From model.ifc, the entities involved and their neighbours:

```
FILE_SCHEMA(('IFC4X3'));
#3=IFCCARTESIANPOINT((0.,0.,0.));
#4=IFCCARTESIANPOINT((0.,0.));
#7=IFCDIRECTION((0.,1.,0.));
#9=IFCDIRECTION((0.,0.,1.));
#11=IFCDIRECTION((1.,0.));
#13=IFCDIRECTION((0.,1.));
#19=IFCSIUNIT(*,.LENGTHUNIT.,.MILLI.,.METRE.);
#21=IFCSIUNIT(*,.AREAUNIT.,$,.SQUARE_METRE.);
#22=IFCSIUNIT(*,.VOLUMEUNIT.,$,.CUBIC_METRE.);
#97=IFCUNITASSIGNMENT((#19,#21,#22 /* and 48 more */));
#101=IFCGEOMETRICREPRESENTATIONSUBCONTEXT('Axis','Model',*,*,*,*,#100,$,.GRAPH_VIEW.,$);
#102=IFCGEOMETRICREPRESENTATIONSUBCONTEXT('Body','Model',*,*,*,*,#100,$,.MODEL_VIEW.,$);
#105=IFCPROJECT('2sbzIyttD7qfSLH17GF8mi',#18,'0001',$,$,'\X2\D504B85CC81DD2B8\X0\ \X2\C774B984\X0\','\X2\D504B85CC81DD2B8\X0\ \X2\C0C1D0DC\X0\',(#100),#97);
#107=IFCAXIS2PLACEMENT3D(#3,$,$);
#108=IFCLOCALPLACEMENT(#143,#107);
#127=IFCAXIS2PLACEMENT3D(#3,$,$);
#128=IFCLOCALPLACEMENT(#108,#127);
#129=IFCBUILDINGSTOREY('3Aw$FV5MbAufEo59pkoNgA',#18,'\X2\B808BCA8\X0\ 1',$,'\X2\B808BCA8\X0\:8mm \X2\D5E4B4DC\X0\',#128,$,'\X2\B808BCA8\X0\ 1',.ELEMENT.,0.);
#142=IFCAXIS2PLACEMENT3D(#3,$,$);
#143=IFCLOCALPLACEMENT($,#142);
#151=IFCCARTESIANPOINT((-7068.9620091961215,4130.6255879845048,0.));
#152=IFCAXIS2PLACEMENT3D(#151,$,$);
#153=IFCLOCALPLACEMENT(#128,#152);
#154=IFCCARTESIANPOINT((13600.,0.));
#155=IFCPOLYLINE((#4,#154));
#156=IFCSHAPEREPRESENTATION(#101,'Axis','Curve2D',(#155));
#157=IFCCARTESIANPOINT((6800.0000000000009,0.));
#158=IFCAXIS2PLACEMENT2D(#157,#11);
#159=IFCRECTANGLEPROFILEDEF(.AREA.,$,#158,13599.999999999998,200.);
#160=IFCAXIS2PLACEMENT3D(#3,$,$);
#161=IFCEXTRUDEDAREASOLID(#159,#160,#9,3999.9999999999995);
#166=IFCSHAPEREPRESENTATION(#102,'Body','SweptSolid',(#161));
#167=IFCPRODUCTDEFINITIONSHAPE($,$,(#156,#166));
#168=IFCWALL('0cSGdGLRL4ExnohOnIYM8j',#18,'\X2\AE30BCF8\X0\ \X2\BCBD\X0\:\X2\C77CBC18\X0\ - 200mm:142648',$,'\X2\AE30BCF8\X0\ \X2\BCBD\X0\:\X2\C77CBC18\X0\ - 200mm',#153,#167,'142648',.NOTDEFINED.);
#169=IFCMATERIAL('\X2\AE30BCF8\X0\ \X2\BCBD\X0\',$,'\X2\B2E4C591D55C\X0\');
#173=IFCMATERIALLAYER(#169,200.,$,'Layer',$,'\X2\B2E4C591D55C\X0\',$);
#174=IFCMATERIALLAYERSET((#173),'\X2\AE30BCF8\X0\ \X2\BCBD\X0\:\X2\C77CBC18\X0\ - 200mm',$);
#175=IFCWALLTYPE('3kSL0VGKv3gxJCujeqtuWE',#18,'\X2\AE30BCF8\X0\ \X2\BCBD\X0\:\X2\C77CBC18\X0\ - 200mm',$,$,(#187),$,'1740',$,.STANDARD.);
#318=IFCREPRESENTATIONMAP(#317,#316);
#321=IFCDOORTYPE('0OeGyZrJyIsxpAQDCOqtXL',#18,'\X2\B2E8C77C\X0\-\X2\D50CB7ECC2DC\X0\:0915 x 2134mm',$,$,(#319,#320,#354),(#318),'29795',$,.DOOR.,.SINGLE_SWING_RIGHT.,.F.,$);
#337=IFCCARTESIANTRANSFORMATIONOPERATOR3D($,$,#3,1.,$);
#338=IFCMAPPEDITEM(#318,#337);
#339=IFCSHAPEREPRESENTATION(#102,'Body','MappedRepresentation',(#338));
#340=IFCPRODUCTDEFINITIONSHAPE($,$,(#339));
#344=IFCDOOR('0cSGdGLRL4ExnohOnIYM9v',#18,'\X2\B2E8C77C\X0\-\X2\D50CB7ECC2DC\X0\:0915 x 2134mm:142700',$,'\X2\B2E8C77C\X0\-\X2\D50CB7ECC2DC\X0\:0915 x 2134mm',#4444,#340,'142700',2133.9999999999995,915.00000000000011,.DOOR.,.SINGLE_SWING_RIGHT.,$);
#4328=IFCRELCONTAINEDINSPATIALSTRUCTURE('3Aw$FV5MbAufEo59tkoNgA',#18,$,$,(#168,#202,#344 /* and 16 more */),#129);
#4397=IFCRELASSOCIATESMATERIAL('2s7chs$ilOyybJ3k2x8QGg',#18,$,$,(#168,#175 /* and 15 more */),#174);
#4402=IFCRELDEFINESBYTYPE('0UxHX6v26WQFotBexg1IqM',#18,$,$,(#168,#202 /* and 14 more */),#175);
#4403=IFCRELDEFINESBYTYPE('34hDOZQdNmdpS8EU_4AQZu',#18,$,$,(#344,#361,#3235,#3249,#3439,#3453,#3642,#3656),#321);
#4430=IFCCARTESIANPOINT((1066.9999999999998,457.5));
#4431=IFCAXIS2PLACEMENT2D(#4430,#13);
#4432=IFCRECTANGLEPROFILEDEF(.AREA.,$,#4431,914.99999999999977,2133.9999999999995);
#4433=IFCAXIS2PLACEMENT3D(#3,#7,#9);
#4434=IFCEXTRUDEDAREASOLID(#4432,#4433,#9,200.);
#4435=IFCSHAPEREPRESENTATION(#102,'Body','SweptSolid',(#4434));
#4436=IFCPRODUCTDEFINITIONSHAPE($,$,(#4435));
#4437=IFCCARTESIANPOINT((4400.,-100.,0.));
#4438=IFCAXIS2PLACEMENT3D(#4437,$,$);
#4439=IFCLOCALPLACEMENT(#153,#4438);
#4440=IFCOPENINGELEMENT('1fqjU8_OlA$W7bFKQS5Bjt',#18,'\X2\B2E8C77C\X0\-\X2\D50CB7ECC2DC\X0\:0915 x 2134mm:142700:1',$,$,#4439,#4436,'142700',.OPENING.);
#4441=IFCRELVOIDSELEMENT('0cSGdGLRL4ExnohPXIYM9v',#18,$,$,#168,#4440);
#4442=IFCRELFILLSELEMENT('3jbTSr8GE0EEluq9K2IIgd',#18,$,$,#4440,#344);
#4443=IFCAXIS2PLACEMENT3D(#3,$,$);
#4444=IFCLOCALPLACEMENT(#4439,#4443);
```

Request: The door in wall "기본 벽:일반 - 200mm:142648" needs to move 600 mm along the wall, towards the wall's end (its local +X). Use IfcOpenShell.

```python
import ifcopenshell
import ifcopenshell.api.geometry
import ifcopenshell.util.placement
import ifcopenshell.util.unit

model = ifcopenshell.open("model.ifc")
unit_scale = ifcopenshell.util.unit.calculate_unit_scale(model)

door = model.by_guid("0cSGdGLRL4ExnohOnIYM9v")
opening = door.FillsVoids[0].RelatingOpeningElement
wall = opening.VoidsElements[0].RelatingBuildingElement

wall_matrix = ifcopenshell.util.placement.get_local_placement(wall.ObjectPlacement)
shift = wall_matrix[:3, 0] * 0.6 / unit_scale
before = ifcopenshell.util.placement.get_local_placement(door.ObjectPlacement)[:3, 3].copy()

# The door is placed relative to its opening, so it follows when the opening moves.
matrix = ifcopenshell.util.placement.get_local_placement(opening.ObjectPlacement)
matrix[:3, 3] += shift
ifcopenshell.api.geometry.edit_object_placement(
    model, product=opening, matrix=matrix, is_si=False, should_transform_children=True
)

after = ifcopenshell.util.placement.get_local_placement(door.ObjectPlacement)[:3, 3]
print("door moved by", (after - before).round(3) + 0.0)

model.write("model_updated.ifc")
```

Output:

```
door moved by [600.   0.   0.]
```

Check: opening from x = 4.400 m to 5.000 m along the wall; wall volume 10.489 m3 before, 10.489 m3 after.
